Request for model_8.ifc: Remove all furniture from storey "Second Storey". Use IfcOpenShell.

First a look at what the model holds.

```python
import ifcopenshell
import ifcopenshell.util.element

model = ifcopenshell.open("model_8.ifc")
print(model.schema)
storey = next(s for s in model.by_type("IfcBuildingStorey") if s.Name == "Second Storey")
furniture = [e for e in ifcopenshell.util.element.get_decomposition(storey) if e.is_a("IfcFurnishingElement")]
seen = {}
for e in furniture:
    element_type = ifcopenshell.util.element.get_type(e)
    name = element_type.Name if element_type not in (None, e) else None
    seen[name] = seen.get(name, 0) + 1
for name, count in sorted(seen.items(), key=str):
    print(count, "x", name)
```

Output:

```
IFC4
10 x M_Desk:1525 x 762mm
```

```python
import ifcopenshell
import ifcopenshell.api.root
import ifcopenshell.util.element

model = ifcopenshell.open("model_8.ifc")

storey = next(s for s in model.by_type("IfcBuildingStorey") if s.Name == "Second Storey")
furniture = [e for e in ifcopenshell.util.element.get_decomposition(storey) if e.is_a("IfcFurnishingElement")]

for e in furniture:
    ifcopenshell.api.root.remove_product(model, product=e)
print(len(furniture), "removed")

model.write("model_8-out.ifc")
```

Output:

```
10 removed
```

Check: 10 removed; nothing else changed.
